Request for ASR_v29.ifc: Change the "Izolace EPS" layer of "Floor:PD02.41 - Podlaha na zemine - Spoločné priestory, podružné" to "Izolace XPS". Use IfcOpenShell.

First a look at what the model holds.

```python
import ifcopenshell
import ifcopenshell.util.element

model = ifcopenshell.open("ASR_v29.ifc")
print(model.schema)
for layer_set in model.by_type("IfcMaterialLayerSet"):
    if layer_set.LayerSetName == "Floor:PD02.41 - Podlaha na zemine - Spoločné priestory, podružné":
        for layer in layer_set.MaterialLayers:
            print(layer.id(), layer.Material and layer.Material.Name, layer.LayerThickness, sep=" | ")
        print(len(ifcopenshell.util.element.get_elements_by_material(model, layer_set)), "elements and types use it")
print(sorted(m.Name for m in model.by_type("IfcMaterial") if m.Name)[:60])
```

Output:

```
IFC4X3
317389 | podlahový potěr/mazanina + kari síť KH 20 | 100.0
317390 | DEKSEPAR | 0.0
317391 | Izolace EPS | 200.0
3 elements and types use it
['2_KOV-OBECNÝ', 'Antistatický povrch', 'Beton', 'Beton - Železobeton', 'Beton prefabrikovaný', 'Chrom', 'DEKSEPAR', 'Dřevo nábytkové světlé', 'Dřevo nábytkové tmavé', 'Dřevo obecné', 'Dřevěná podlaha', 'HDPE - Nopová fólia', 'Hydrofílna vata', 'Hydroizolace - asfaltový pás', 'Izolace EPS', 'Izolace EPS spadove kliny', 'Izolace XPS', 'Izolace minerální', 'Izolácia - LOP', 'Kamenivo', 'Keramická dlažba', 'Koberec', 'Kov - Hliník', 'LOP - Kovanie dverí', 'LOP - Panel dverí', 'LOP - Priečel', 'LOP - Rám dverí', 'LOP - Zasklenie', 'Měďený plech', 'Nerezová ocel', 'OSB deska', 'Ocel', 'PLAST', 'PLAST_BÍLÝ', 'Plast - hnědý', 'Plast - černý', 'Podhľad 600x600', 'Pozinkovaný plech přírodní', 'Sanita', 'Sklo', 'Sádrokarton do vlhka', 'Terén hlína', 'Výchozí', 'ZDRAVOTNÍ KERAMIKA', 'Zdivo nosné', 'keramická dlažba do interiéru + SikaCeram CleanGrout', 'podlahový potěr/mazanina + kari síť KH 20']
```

```python
import ifcopenshell
import ifcopenshell.api.material

model = ifcopenshell.open("ASR_v29.ifc")

layer_set = next(s for s in model.by_type("IfcMaterialLayerSet") if s.LayerSetName == "Floor:PD02.41 - Podlaha na zemine - Spoločné priestory, podružné")
layer = next(l for l in layer_set.MaterialLayers if l.Material and l.Material.Name == "Izolace EPS")
material = next(m for m in model.by_type("IfcMaterial") if m.Name == "Izolace XPS")

# Point this one layer at the other material; renaming the old one would change it everywhere.
ifcopenshell.api.material.edit_layer(model, layer=layer, attributes={"Name": material.Name}, material=material)

print([l.Material.Name if l.Material else None for l in layer_set.MaterialLayers])

model.write("ASR_v29-out.ifc")
```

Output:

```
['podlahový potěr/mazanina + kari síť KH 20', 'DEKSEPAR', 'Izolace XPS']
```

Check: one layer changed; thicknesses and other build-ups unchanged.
